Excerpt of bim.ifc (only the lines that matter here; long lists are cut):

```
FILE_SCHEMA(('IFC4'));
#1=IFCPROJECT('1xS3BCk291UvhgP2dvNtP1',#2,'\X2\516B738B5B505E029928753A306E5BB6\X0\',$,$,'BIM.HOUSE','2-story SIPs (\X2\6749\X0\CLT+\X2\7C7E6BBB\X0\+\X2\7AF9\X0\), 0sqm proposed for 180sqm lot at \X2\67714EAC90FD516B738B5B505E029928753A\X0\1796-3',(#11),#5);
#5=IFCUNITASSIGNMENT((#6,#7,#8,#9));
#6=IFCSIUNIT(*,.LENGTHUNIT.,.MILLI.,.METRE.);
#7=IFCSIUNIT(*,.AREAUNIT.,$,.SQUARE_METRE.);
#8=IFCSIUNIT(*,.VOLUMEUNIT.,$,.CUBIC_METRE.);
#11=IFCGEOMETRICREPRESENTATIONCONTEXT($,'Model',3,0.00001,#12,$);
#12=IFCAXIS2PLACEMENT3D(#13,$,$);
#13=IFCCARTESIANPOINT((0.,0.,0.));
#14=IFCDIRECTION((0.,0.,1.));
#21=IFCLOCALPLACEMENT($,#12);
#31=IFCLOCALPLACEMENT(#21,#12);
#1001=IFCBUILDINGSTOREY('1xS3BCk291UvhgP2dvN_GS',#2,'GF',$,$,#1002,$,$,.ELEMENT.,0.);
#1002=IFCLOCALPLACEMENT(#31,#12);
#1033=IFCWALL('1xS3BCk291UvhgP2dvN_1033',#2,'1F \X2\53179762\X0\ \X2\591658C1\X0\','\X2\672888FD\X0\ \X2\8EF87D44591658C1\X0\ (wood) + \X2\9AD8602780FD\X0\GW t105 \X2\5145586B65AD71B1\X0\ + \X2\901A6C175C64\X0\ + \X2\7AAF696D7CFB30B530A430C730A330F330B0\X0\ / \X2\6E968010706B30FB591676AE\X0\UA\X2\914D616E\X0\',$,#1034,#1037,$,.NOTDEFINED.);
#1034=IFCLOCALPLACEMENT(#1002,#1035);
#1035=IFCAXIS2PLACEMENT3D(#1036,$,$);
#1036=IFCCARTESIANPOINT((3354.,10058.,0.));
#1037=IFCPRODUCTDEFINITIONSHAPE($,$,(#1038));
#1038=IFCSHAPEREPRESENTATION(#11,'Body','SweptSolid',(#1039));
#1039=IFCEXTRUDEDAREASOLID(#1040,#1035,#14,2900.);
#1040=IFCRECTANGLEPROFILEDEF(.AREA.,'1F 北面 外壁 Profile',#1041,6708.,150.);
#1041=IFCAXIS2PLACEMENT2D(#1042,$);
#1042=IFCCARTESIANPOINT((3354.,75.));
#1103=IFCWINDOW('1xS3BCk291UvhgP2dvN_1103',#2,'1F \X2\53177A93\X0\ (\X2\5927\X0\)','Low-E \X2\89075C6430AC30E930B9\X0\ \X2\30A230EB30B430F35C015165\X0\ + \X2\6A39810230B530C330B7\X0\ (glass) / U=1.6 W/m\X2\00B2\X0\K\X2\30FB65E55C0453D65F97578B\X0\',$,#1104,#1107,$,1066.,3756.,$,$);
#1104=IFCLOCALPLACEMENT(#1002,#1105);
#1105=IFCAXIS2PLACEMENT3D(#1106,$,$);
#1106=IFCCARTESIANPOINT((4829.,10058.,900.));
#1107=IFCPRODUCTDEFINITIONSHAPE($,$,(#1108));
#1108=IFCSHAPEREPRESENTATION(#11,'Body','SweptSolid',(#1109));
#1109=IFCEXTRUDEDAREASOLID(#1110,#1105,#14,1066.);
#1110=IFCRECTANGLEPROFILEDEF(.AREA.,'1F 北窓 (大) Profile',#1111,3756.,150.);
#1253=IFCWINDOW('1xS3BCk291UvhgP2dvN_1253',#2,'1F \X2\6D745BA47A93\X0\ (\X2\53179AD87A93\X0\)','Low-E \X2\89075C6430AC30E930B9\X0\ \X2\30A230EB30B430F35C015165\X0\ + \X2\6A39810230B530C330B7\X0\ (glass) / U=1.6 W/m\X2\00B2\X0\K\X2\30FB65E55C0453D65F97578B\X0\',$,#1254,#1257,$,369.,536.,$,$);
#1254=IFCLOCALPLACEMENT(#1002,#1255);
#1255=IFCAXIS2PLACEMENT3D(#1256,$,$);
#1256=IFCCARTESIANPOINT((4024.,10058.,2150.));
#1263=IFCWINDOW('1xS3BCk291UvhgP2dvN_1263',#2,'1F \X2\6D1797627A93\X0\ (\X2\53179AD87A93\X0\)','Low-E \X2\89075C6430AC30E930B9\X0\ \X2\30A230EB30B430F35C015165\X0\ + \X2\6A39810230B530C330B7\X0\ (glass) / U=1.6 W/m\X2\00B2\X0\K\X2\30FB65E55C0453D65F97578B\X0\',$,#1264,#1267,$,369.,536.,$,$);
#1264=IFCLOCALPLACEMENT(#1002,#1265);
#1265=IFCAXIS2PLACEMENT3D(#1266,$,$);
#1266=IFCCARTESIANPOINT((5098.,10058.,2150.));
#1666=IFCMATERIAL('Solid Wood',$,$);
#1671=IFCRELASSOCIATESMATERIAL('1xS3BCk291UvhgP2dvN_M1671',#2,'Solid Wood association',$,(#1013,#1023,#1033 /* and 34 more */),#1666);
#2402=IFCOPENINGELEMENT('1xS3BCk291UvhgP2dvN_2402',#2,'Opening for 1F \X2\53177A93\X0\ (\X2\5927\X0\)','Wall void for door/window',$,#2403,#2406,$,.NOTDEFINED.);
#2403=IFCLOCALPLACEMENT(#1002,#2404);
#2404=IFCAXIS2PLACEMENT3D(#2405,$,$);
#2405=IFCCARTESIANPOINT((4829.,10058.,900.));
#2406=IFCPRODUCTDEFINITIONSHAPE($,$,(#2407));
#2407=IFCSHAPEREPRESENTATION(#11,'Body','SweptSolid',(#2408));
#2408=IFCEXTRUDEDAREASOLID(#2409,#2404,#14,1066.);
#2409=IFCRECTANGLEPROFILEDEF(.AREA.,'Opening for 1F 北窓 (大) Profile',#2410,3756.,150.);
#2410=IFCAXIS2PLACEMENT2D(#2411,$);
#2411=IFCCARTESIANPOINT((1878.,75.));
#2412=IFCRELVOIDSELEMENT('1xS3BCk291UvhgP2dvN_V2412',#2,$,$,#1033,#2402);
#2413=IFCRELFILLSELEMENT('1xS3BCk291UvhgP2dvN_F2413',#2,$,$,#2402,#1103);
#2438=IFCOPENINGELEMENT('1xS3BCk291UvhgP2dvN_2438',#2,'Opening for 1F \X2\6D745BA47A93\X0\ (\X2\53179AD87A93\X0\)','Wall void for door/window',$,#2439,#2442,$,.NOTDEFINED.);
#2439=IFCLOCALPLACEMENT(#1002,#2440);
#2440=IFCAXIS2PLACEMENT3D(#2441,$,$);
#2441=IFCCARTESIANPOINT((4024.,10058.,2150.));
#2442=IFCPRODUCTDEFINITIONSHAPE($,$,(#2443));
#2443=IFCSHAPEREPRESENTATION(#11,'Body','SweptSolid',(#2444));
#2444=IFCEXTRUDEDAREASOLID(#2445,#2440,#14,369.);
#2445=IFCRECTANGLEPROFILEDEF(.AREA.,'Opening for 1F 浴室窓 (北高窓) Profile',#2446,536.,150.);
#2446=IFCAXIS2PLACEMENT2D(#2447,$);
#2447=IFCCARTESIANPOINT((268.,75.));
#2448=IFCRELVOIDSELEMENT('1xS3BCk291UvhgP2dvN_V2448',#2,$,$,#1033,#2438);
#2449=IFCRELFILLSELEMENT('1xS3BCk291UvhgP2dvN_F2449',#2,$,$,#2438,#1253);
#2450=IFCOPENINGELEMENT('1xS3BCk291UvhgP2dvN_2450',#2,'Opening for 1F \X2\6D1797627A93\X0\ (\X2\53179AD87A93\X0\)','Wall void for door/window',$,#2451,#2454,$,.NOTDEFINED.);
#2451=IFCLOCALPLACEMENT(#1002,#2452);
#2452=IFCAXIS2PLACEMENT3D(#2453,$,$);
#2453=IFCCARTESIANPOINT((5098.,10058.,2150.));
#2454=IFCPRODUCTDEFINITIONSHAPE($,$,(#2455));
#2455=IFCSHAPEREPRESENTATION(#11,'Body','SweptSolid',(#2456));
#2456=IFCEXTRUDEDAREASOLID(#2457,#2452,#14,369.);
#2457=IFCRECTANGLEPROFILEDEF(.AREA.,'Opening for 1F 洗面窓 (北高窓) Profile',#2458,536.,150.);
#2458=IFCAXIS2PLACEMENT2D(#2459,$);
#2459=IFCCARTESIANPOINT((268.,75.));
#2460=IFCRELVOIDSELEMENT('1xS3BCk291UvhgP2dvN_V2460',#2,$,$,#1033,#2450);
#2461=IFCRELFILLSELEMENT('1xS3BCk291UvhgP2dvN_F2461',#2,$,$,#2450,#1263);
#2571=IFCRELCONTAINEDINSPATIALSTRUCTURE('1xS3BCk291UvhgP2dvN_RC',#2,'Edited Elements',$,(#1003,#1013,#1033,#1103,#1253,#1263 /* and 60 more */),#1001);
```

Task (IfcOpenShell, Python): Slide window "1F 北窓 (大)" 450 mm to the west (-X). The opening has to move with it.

```python
import ifcopenshell
import ifcopenshell.api.geometry
import ifcopenshell.util.placement

model = ifcopenshell.open("bim.ifc")

window = model.by_guid("1xS3BCk291UvhgP2dvN_1103")
opening = window.FillsVoids[0].RelatingOpeningElement
wall = opening.VoidsElements[0].RelatingBuildingElement

wall_matrix = ifcopenshell.util.placement.get_local_placement(wall.ObjectPlacement)
shift = wall_matrix[:3, 0] * -450.0
before = ifcopenshell.util.placement.get_local_placement(window.ObjectPlacement)[:3, 3].copy()

# The window is not placed relative to its opening, so move both.
for product in (opening, window):
    matrix = ifcopenshell.util.placement.get_local_placement(product.ObjectPlacement)
    matrix[:3, 3] += shift
    ifcopenshell.api.geometry.edit_object_placement(model, product=product, matrix=matrix, is_si=False)

after = ifcopenshell.util.placement.get_local_placement(window.ObjectPlacement)[:3, 3]
print("window moved by", (after - before).round(3) + 0.0)

model.write("bim_edited.ifc")
```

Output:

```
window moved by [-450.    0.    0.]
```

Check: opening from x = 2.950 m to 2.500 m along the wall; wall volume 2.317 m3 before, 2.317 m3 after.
